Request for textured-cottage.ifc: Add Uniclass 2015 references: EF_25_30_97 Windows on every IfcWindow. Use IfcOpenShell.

First a look at what the model holds.

```python
import ifcopenshell

model = ifcopenshell.open("textured-cottage.ifc")
print(model.schema)
print("classifications:", [c.Name for c in model.by_type("IfcClassification")])
for ifc_class in ("IfcDoor", "IfcRoof", "IfcStair", "IfcWall", "IfcWindow"):
    print(ifc_class, len(model.by_type(ifc_class)))
```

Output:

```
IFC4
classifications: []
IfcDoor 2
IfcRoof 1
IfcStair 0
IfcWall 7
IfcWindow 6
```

```python
import ifcopenshell
import ifcopenshell.api.classification

model = ifcopenshell.open("textured-cottage.ifc")

system = ifcopenshell.api.classification.add_classification(model, classification="Uniclass 2015")

codes = {
    "IfcWindow": ("EF_25_30_97", "Windows"),
}
for ifc_class, (code, name) in codes.items():
    products = model.by_type(ifc_class)
    ifcopenshell.api.classification.add_reference(
        model, products=products, classification=system, identification=code, name=name
    )
    print(code, len(products))

model.write("textured-cottage_rev.ifc")
```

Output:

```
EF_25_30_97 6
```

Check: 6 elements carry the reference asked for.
